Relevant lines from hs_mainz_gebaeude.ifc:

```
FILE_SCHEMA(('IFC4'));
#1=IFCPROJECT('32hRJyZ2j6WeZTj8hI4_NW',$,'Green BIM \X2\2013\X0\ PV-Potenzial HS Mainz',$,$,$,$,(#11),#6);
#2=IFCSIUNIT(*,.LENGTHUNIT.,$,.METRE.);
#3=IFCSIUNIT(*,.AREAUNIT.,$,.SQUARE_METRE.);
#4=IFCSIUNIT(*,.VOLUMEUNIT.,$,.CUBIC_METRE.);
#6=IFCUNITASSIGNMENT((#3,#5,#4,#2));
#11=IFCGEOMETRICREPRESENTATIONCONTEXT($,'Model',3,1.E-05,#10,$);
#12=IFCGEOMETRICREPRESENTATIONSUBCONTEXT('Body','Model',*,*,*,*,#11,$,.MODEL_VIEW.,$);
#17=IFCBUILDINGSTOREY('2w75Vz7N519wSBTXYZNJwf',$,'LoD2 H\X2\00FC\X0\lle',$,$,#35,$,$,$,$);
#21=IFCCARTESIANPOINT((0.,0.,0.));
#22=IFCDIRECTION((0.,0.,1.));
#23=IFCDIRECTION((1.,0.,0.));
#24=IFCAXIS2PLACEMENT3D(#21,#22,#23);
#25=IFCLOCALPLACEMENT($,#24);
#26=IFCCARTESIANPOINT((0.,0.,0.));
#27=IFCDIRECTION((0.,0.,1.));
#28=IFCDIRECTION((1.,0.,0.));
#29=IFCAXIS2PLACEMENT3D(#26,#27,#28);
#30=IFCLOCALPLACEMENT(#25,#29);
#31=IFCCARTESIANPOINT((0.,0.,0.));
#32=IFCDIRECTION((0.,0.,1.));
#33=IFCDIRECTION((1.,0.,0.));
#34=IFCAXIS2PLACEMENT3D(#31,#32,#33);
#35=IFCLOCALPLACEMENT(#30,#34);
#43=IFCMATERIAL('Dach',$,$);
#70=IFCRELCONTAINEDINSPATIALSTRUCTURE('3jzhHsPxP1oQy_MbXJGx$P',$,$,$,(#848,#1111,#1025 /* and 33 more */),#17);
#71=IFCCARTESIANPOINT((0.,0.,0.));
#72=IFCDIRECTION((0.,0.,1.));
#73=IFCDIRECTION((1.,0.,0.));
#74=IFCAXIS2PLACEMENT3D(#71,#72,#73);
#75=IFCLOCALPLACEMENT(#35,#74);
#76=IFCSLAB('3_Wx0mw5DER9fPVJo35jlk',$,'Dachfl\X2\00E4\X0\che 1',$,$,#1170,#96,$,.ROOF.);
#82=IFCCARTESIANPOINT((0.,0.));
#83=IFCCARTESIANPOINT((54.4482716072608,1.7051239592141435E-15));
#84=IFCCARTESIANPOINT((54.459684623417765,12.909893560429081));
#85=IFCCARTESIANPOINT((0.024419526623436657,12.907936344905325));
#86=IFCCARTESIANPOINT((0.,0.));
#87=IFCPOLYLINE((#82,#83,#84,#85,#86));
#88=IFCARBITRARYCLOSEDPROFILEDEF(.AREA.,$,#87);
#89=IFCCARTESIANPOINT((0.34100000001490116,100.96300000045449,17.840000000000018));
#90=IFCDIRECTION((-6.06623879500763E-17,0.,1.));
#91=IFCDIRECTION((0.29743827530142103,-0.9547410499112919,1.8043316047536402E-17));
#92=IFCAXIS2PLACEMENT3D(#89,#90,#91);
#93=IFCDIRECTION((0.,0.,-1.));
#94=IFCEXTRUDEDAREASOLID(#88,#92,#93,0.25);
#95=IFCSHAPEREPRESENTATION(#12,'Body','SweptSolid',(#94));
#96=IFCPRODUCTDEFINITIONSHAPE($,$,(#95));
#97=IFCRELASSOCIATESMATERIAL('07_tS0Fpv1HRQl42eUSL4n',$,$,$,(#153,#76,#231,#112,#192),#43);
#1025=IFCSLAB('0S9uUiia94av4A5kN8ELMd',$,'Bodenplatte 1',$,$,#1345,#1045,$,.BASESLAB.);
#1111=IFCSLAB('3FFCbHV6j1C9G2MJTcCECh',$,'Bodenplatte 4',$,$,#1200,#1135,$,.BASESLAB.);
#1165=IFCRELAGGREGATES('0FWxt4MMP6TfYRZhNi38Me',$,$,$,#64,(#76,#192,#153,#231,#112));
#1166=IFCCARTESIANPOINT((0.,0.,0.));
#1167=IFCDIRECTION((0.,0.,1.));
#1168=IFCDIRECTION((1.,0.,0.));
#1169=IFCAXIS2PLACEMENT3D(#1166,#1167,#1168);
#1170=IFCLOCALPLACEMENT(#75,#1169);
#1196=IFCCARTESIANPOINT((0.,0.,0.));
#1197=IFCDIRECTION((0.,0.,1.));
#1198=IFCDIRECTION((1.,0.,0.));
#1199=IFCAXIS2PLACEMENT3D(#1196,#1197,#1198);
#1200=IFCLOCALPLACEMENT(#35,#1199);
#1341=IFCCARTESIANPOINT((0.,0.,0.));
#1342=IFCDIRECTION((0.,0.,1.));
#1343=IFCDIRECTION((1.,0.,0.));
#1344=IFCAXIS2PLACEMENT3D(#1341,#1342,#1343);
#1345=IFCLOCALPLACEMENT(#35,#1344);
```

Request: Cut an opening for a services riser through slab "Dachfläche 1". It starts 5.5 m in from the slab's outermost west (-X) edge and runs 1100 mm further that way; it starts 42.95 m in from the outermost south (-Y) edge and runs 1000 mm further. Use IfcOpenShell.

```python
import numpy as np
import ifcopenshell
import ifcopenshell.api.feature
import ifcopenshell.api.geometry
import ifcopenshell.api.root
import ifcopenshell.geom
import ifcopenshell.util.placement
import ifcopenshell.util.representation
import ifcopenshell.util.shape
import ifcopenshell.util.unit

model = ifcopenshell.open("hs_mainz_gebaeude.ifc")
unit_scale = ifcopenshell.util.unit.calculate_unit_scale(model)
settings = ifcopenshell.geom.settings()


def volume(element):
    """Net volume in cubic metres, openings subtracted."""
    shape = ifcopenshell.geom.create_shape(settings, element)
    return ifcopenshell.util.shape.get_volume(shape.geometry)


slab = model.by_guid("3_Wx0mw5DER9fPVJo35jlk")
before = volume(slab)

# Extent in the slab's own axes, in metres. The edges named are its -X and -Y sides.
slab_shape = ifcopenshell.geom.create_shape(settings, slab)
vertices = ifcopenshell.util.shape.get_vertices(slab_shape.geometry)
x_min, y_min, bottom = vertices.min(axis=0)
top = vertices[:, 2].max()

opening = ifcopenshell.api.root.create_entity(model, ifc_class="IfcOpeningElement", name="Services riser opening", predefined_type="OPENING")
context = ifcopenshell.util.representation.get_context(model, "Model", "Body", "MODEL_VIEW")
width, depth = 1.1, 1
outline = [(0.0, 0.0), (width, 0.0), (width, depth), (0.0, depth), (0.0, 0.0)]
# Overshoot both faces by 50 mm so the cut is clean.
shape = ifcopenshell.api.geometry.add_slab_representation(
    model, context=context, depth=top - bottom + 0.1, polyline=outline
)
ifcopenshell.api.geometry.assign_representation(model, product=opening, representation=shape)

matrix = ifcopenshell.util.placement.get_local_placement(slab.ObjectPlacement)
matrix[:, 3] = matrix @ np.append(np.array([x_min + 5.5, y_min + 42.95, bottom - 0.05]) / unit_scale, 1.0)
ifcopenshell.api.geometry.edit_object_placement(model, product=opening, matrix=matrix, is_si=False)
ifcopenshell.api.feature.add_feature(model, feature=opening, element=slab)

after = volume(slab)

print(f"slab volume {before:.3f} -> {after:.3f} m3")

model.write("hs_mainz_gebaeude_v2.ifc")
```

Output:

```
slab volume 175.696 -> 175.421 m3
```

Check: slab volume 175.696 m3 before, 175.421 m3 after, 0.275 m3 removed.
